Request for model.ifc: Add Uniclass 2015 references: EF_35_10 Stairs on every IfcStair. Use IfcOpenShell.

First a look at what the model holds.

```python
import ifcopenshell

model = ifcopenshell.open("model.ifc")
print(model.schema)
print("classifications:", [c.Name for c in model.by_type("IfcClassification")])
for ifc_class in ("IfcDoor", "IfcRoof", "IfcStair", "IfcWall", "IfcWindow"):
    print(ifc_class, len(model.by_type(ifc_class)))
```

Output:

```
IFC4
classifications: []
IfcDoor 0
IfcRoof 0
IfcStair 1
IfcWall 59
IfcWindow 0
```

```python
import ifcopenshell
import ifcopenshell.api.classification

model = ifcopenshell.open("model.ifc")

system = ifcopenshell.api.classification.add_classification(model, classification="Uniclass 2015")

codes = {
    "IfcStair": ("EF_35_10", "Stairs"),
}
for ifc_class, (code, name) in codes.items():
    products = model.by_type(ifc_class)
    ifcopenshell.api.classification.add_reference(
        model, products=products, classification=system, identification=code, name=name
    )
    print(code, len(products))

model.write("model_edited.ifc")
```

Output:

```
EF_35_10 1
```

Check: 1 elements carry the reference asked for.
